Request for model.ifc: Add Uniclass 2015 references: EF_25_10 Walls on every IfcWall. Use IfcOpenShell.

First a look at what the model holds.

```python
import ifcopenshell

model = ifcopenshell.open("model.ifc")
print(model.schema)
print("classifications:", [c.Name for c in model.by_type("IfcClassification")])
for ifc_class in ("IfcDoor", "IfcRoof", "IfcStair", "IfcWall", "IfcWindow"):
    print(ifc_class, len(model.by_type(ifc_class)))
```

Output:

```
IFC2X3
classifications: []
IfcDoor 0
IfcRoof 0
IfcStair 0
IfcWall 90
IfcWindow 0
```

```python
import ifcopenshell
import ifcopenshell.api.classification

model = ifcopenshell.open("model.ifc")

# IFC2X3 requires Source and Edition and has no link from the project to the system.
system = model.create_entity("IfcClassification", Source="NBS", Edition="2015", Name="Uniclass 2015")

codes = {
    "IfcWall": ("EF_25_10", "Walls"),
}
for ifc_class, (code, name) in codes.items():
    products = model.by_type(ifc_class)
    ifcopenshell.api.classification.add_reference(
        model, products=products, classification=system, identification=code, name=name
    )
    print(code, len(products))

model.write("model_rev.ifc")
```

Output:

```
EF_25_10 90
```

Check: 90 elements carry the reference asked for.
